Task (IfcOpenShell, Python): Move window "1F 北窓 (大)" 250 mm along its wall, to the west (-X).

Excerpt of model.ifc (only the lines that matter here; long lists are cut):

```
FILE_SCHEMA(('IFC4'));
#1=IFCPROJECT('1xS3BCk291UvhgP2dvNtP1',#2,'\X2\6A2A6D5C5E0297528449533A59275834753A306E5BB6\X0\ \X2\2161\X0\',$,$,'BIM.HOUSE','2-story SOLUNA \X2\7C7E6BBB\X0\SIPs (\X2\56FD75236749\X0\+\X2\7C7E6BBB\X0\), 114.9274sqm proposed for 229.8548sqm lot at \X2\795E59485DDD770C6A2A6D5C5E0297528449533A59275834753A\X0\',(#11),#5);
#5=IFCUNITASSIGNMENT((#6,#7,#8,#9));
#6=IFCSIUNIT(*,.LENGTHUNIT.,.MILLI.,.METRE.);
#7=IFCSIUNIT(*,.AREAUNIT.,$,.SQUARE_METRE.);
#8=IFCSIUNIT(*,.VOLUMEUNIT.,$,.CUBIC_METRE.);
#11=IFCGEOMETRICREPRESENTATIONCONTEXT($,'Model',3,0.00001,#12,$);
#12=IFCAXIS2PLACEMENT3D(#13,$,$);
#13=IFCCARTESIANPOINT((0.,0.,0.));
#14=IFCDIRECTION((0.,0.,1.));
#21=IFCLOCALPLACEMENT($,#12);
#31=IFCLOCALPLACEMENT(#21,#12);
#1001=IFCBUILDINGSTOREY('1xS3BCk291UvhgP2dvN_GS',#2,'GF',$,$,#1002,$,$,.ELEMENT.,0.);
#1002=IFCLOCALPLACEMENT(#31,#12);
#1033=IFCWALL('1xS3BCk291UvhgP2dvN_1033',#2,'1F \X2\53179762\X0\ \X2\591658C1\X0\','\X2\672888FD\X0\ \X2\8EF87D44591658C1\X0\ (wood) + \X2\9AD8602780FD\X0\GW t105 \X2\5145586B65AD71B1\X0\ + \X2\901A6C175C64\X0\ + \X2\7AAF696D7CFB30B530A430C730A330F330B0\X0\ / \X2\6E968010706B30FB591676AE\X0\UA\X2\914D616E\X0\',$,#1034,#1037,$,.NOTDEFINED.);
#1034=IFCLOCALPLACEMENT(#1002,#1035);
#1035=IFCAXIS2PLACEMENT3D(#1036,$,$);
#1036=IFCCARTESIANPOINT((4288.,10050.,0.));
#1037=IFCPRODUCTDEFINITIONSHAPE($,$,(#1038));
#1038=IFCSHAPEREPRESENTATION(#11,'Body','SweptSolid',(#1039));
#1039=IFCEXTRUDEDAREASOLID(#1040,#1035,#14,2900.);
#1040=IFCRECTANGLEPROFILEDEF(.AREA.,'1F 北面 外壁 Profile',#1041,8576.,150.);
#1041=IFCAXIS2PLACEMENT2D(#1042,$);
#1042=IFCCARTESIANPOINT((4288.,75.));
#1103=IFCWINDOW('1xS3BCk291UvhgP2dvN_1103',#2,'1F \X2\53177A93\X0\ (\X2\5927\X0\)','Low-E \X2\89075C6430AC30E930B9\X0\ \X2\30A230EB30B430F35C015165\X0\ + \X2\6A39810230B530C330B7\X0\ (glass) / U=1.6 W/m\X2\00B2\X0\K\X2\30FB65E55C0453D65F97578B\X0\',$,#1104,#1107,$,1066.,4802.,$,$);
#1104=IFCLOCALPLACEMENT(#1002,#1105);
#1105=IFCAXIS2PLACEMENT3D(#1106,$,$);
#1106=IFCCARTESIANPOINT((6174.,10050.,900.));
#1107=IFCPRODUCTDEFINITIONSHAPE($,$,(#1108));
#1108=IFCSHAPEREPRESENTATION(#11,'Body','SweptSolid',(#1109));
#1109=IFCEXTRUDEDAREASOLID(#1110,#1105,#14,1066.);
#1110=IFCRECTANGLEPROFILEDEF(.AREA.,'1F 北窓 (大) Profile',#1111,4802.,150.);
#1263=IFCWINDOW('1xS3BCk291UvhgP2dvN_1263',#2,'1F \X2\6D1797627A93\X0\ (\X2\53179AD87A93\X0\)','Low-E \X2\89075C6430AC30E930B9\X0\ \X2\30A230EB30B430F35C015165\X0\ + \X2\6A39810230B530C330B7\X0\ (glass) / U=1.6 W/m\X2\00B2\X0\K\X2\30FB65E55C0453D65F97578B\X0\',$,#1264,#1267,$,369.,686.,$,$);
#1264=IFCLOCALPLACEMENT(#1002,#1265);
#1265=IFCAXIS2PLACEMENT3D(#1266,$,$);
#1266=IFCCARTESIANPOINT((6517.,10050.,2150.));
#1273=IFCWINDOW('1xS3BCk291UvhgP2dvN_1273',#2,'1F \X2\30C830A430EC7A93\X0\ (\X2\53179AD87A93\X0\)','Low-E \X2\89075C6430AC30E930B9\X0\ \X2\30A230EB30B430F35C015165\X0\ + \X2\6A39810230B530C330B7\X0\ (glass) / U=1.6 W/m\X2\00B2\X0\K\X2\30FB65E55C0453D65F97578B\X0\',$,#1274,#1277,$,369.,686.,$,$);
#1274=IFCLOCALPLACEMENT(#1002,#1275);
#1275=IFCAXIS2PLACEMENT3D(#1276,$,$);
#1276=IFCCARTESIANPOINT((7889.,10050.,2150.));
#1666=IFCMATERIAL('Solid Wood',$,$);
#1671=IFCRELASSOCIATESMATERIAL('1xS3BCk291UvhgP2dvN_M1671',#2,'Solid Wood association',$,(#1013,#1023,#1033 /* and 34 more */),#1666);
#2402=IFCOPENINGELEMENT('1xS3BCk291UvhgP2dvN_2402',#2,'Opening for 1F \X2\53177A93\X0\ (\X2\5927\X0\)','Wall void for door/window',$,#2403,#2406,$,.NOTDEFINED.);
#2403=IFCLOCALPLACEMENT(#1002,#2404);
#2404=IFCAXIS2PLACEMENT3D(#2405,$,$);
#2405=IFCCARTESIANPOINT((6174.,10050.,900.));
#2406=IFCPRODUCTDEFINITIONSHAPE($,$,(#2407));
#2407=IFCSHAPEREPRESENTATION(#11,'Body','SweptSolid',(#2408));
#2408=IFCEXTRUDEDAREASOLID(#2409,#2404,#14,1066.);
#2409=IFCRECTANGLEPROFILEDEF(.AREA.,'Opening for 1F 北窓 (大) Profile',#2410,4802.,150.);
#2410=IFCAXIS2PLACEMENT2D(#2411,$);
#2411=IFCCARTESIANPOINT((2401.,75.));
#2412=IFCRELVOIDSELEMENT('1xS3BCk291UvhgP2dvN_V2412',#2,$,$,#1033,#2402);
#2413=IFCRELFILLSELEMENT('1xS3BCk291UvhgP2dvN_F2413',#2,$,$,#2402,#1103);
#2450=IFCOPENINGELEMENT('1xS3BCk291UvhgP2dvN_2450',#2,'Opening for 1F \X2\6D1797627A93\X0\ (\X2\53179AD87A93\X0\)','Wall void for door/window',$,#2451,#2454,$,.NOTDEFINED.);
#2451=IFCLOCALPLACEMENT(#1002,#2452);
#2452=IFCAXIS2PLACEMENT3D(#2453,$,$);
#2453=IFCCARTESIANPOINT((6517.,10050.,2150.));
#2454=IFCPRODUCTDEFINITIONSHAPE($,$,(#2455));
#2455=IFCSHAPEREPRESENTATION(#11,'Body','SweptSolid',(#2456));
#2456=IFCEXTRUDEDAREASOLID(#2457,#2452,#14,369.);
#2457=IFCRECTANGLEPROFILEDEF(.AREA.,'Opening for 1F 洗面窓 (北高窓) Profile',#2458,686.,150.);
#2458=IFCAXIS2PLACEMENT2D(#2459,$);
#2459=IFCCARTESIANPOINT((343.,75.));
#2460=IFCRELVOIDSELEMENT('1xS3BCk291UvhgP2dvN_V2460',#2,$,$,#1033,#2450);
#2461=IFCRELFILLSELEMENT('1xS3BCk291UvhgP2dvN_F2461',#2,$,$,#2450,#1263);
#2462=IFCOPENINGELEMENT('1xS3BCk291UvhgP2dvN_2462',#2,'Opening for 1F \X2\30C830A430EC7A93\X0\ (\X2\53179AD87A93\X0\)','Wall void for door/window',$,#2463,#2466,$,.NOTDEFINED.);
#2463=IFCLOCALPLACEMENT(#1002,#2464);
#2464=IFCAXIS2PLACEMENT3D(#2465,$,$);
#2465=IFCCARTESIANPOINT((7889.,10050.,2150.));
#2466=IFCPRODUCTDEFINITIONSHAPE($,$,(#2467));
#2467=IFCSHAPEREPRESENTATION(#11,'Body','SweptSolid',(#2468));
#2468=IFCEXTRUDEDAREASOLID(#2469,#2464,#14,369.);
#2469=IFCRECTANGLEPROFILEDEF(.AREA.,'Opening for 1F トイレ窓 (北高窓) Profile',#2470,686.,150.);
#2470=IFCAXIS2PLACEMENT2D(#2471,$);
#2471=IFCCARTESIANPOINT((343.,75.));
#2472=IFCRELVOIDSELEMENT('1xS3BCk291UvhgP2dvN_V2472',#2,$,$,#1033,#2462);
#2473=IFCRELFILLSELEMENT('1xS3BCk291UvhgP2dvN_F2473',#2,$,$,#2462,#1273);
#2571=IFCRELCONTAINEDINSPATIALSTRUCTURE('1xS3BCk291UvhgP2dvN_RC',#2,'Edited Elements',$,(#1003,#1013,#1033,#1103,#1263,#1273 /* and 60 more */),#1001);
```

```python
import ifcopenshell
import ifcopenshell.api.geometry
import ifcopenshell.util.placement
import ifcopenshell.util.unit

model = ifcopenshell.open("model.ifc")
unit_scale = ifcopenshell.util.unit.calculate_unit_scale(model)

window = model.by_guid("1xS3BCk291UvhgP2dvN_1103")
opening = window.FillsVoids[0].RelatingOpeningElement
wall = opening.VoidsElements[0].RelatingBuildingElement

wall_matrix = ifcopenshell.util.placement.get_local_placement(wall.ObjectPlacement)
shift = wall_matrix[:3, 0] * -0.25 / unit_scale
before = ifcopenshell.util.placement.get_local_placement(window.ObjectPlacement)[:3, 3].copy()

# The window is not placed relative to its opening, so move both.
for product in (opening, window):
    matrix = ifcopenshell.util.placement.get_local_placement(product.ObjectPlacement)
    matrix[:3, 3] += shift
    ifcopenshell.api.geometry.edit_object_placement(model, product=product, matrix=matrix, is_si=False)

after = ifcopenshell.util.placement.get_local_placement(window.ObjectPlacement)[:3, 3]
print("window moved by", (after - before).round(3) + 0.0)

model.write("model_v2.ifc")
```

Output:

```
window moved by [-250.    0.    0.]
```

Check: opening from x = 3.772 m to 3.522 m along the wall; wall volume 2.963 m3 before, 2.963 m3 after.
